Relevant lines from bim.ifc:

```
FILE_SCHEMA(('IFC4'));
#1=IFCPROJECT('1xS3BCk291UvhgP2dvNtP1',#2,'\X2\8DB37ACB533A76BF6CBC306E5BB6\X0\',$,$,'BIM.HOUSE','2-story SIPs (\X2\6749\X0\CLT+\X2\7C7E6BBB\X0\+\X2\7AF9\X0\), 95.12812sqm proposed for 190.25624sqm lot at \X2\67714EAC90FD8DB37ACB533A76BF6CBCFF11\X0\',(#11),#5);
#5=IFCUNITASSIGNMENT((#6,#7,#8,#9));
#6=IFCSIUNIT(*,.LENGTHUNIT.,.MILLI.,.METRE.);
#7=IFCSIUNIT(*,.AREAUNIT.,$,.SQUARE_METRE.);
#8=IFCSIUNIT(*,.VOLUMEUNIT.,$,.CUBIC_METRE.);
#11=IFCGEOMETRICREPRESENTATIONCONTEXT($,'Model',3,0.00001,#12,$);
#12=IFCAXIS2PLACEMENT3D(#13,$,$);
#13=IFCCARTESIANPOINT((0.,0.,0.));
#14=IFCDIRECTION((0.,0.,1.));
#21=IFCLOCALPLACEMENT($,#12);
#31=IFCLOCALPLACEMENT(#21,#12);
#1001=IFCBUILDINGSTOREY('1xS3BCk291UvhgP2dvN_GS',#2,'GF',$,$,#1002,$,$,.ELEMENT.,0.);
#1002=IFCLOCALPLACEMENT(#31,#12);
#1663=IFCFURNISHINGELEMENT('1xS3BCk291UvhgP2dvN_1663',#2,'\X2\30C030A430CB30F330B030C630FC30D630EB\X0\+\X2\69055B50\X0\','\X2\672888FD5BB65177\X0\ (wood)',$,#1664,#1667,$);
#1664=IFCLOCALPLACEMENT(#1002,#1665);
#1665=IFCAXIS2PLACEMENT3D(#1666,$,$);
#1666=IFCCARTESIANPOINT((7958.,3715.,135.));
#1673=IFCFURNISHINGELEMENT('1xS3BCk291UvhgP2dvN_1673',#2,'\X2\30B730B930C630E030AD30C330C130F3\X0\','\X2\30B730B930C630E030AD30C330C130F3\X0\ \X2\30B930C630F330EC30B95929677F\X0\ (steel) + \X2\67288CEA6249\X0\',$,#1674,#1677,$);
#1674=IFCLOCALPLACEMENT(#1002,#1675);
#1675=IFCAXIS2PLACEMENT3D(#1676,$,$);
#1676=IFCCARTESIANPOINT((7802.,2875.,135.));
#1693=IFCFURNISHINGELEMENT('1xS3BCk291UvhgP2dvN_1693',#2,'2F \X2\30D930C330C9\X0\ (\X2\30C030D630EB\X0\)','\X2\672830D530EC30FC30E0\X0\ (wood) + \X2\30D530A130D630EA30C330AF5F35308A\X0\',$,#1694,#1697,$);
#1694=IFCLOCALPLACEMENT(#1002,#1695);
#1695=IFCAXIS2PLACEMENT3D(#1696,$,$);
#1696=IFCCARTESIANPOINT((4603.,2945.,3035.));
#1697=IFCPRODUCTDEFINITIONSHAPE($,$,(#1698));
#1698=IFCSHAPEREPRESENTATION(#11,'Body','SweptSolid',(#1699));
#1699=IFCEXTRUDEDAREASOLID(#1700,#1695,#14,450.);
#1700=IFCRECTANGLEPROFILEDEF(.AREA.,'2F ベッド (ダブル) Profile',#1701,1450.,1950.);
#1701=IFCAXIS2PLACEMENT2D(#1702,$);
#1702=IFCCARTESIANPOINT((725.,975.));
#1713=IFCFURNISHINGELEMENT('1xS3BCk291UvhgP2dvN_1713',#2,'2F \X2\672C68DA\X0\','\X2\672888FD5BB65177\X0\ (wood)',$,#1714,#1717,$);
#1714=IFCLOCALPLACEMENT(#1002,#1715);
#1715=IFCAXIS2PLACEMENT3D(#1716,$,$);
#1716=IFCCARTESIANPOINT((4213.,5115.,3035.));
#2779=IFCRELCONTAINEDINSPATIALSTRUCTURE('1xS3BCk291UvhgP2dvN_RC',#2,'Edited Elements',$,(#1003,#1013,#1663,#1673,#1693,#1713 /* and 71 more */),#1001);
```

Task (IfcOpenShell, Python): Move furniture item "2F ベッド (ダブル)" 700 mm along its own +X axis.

```python
import ifcopenshell
import ifcopenshell.api.geometry
import ifcopenshell.util.placement

model = ifcopenshell.open("bim.ifc")

item = model.by_guid("1xS3BCk291UvhgP2dvN_1693")
matrix = ifcopenshell.util.placement.get_local_placement(item.ObjectPlacement)
matrix[:3, 3] += matrix[:3, 0] * 700.0
ifcopenshell.api.geometry.edit_object_placement(model, product=item, matrix=matrix, is_si=False)

print(ifcopenshell.util.placement.get_local_placement(item.ObjectPlacement).round(3) + 0.0)

model.write("bim_rev.ifc")
```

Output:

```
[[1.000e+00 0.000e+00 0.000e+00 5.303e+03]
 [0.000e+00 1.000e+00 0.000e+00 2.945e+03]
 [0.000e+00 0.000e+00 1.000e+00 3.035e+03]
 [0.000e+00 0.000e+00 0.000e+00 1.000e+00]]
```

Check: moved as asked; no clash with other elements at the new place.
